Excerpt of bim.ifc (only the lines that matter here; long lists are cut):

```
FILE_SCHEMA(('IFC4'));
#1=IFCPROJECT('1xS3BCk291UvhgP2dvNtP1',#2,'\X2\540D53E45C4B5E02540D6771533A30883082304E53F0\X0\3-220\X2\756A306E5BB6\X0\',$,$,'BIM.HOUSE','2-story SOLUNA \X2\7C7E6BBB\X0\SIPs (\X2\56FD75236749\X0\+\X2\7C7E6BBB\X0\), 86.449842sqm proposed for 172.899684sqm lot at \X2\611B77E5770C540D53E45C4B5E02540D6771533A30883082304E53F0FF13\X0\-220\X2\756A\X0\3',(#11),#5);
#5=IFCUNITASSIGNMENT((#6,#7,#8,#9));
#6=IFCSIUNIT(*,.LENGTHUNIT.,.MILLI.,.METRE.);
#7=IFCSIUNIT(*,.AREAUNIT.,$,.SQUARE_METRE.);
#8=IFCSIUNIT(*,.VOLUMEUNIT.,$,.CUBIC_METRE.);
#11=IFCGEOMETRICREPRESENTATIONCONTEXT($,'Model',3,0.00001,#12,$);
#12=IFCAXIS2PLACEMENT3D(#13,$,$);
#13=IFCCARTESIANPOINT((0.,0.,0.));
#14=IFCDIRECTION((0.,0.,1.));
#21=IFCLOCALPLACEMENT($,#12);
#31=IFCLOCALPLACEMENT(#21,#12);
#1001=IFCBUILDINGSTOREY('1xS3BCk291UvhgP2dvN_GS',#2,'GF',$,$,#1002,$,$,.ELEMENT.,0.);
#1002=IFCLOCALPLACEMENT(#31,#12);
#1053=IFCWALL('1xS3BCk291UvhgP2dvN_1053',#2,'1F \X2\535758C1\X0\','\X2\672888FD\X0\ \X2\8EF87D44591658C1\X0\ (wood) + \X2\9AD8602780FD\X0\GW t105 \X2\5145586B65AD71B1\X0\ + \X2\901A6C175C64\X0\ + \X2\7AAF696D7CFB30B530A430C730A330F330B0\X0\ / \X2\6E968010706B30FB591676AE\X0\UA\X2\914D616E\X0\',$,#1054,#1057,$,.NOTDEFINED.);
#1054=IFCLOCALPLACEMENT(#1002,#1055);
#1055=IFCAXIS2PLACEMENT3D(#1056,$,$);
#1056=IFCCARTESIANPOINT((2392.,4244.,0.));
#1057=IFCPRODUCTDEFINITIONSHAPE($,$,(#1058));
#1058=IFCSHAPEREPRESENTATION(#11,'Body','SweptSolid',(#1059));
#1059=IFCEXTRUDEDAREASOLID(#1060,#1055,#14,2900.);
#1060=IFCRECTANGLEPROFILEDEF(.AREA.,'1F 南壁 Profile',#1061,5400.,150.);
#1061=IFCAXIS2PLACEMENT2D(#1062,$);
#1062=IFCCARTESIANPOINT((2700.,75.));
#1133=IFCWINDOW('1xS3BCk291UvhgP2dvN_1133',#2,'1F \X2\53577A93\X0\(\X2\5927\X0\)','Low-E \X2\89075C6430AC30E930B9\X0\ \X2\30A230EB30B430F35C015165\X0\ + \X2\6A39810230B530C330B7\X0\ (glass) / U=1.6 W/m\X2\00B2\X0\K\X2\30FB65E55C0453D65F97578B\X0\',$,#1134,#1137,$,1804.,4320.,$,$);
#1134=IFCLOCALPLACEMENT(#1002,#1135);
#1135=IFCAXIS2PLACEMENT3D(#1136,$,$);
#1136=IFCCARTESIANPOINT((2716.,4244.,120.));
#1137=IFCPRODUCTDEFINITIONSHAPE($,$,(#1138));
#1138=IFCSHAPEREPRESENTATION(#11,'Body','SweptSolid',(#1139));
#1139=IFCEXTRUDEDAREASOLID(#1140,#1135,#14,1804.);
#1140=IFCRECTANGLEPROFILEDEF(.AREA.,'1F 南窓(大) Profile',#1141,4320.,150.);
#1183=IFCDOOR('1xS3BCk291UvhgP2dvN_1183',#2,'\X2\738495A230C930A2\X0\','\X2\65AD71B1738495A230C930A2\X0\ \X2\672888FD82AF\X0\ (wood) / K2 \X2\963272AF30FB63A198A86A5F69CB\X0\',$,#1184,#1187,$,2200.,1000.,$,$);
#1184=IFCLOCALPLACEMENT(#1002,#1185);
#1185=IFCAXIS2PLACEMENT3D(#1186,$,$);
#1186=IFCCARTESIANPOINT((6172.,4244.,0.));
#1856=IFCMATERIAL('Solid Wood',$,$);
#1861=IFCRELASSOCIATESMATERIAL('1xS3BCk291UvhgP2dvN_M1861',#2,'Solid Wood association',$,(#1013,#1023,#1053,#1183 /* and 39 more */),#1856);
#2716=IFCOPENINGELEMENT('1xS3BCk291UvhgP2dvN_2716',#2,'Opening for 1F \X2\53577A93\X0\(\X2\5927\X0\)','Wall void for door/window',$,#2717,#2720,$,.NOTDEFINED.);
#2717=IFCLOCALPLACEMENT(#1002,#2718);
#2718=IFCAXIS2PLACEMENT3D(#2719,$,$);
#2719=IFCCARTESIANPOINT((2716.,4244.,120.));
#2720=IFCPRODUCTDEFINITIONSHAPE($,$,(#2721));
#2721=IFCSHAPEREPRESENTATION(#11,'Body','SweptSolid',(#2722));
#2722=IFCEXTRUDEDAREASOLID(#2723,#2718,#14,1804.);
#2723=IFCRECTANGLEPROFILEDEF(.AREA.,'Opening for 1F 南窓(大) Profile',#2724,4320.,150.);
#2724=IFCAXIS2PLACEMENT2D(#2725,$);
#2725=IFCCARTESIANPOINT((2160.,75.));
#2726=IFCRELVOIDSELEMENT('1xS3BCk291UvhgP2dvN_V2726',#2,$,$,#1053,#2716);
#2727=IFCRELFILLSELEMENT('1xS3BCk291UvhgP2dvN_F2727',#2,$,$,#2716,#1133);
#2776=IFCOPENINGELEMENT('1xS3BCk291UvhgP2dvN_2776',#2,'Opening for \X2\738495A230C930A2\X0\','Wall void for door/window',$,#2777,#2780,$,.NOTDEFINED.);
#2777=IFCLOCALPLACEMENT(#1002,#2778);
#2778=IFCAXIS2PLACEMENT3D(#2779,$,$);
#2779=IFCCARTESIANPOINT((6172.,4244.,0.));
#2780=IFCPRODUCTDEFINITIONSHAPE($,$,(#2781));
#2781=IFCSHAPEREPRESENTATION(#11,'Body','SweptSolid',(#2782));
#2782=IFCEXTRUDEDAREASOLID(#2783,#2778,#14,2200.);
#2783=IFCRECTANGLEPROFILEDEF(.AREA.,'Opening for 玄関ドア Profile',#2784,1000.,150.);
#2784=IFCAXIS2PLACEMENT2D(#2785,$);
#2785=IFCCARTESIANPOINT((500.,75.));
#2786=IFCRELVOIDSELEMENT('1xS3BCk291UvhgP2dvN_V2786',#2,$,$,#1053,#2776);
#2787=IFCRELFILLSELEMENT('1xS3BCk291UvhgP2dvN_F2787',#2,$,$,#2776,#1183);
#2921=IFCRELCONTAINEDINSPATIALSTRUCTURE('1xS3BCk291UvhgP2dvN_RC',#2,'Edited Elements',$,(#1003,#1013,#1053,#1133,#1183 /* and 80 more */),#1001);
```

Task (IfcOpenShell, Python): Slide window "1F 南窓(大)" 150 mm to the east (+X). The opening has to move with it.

```python
import ifcopenshell
import ifcopenshell.api.geometry
import ifcopenshell.util.placement

model = ifcopenshell.open("bim.ifc")

window = model.by_guid("1xS3BCk291UvhgP2dvN_1133")
opening = window.FillsVoids[0].RelatingOpeningElement
wall = opening.VoidsElements[0].RelatingBuildingElement

wall_matrix = ifcopenshell.util.placement.get_local_placement(wall.ObjectPlacement)
shift = wall_matrix[:3, 0] * 150.0
before = ifcopenshell.util.placement.get_local_placement(window.ObjectPlacement)[:3, 3].copy()

# The window is not placed relative to its opening, so move both.
for product in (opening, window):
    matrix = ifcopenshell.util.placement.get_local_placement(product.ObjectPlacement)
    matrix[:3, 3] += shift
    ifcopenshell.api.geometry.edit_object_placement(model, product=product, matrix=matrix, is_si=False)

after = ifcopenshell.util.placement.get_local_placement(window.ObjectPlacement)[:3, 3]
print("window moved by", (after - before).round(3) + 0.0)

model.write("bim-out.ifc")
```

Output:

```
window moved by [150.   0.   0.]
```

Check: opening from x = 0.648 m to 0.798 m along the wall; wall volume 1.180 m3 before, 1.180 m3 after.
